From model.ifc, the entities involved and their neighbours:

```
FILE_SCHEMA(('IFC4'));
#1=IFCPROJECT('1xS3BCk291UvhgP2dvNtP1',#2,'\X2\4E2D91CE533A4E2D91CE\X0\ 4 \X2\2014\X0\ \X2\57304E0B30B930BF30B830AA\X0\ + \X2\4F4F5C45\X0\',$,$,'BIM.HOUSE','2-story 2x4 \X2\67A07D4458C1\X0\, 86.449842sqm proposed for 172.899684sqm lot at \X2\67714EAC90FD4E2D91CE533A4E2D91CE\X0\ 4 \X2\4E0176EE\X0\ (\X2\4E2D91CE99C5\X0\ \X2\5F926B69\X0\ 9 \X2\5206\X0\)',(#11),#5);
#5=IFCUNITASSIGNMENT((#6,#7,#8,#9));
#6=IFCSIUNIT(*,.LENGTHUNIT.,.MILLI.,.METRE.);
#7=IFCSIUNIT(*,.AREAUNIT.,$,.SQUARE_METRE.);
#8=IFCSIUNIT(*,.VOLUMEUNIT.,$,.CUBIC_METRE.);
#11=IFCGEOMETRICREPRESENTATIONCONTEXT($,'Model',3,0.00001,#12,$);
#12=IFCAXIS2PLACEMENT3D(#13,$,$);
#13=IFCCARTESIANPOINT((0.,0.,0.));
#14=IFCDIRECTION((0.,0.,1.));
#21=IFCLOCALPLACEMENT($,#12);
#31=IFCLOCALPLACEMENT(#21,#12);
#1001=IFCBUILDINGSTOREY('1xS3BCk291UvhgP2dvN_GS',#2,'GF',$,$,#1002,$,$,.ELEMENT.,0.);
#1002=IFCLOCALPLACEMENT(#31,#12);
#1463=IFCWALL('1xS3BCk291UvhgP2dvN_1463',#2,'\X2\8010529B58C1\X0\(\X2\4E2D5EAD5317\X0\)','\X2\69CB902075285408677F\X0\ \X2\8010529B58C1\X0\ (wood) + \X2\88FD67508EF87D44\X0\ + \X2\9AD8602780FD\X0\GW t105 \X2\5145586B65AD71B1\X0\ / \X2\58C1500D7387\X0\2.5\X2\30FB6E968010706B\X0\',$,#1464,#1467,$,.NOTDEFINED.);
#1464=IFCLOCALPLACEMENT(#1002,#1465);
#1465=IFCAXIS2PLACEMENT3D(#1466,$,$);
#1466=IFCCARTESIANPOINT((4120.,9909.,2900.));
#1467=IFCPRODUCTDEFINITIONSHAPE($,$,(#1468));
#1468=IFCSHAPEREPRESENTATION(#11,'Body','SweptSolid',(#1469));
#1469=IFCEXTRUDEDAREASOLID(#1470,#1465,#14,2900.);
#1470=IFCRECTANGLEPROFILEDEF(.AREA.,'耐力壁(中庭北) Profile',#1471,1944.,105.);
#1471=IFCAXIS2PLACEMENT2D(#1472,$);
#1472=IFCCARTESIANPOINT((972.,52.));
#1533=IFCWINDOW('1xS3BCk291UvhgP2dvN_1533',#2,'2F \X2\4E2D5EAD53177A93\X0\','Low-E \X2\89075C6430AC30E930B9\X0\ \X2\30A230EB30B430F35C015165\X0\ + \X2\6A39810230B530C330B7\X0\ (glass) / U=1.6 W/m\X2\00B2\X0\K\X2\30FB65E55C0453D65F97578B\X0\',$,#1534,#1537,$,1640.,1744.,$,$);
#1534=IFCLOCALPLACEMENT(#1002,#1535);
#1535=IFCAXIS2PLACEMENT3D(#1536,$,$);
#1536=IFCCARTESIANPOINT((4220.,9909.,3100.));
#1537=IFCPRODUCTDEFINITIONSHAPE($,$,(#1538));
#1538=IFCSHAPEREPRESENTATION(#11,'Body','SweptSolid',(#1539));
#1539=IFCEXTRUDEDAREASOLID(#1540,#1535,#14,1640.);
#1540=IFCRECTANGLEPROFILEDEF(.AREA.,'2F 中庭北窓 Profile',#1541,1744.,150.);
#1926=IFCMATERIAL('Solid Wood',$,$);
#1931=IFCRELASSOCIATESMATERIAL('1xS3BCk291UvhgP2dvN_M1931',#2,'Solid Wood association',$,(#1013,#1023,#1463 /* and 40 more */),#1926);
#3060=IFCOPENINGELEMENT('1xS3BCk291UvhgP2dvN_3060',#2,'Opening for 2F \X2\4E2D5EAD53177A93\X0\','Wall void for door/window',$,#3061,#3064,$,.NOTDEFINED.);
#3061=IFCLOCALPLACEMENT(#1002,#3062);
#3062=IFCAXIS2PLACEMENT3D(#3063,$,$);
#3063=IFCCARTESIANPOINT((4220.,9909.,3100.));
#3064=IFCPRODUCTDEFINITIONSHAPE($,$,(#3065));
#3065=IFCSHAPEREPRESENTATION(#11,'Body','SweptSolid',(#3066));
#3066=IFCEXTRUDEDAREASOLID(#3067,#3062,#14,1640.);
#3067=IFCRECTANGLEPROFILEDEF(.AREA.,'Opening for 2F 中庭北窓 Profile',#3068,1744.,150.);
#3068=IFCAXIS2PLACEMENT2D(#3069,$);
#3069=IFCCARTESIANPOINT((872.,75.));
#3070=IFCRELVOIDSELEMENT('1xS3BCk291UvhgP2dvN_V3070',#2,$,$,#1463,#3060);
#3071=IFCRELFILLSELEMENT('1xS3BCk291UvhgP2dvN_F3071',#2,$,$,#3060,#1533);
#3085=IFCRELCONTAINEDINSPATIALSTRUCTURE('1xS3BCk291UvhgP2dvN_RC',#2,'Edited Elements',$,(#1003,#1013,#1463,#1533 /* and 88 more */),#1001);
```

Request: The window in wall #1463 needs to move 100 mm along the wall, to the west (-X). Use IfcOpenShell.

```python
import ifcopenshell
import ifcopenshell.api.geometry
import ifcopenshell.util.placement
import ifcopenshell.util.unit

model = ifcopenshell.open("model.ifc")
unit_scale = ifcopenshell.util.unit.calculate_unit_scale(model)

window = model.by_id(1533)
opening = window.FillsVoids[0].RelatingOpeningElement
wall = opening.VoidsElements[0].RelatingBuildingElement

wall_matrix = ifcopenshell.util.placement.get_local_placement(wall.ObjectPlacement)
shift = wall_matrix[:3, 0] * -0.1 / unit_scale
before = ifcopenshell.util.placement.get_local_placement(window.ObjectPlacement)[:3, 3].copy()

# The window is not placed relative to its opening, so move both.
for product in (opening, window):
    matrix = ifcopenshell.util.placement.get_local_placement(product.ObjectPlacement)
    matrix[:3, 3] += shift
    ifcopenshell.api.geometry.edit_object_placement(model, product=product, matrix=matrix, is_si=False)

after = ifcopenshell.util.placement.get_local_placement(window.ObjectPlacement)[:3, 3]
print("window moved by", (after - before).round(3) + 0.0)

model.write("model_edited.ifc")
```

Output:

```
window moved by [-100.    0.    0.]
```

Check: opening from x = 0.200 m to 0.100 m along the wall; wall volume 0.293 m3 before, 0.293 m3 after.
